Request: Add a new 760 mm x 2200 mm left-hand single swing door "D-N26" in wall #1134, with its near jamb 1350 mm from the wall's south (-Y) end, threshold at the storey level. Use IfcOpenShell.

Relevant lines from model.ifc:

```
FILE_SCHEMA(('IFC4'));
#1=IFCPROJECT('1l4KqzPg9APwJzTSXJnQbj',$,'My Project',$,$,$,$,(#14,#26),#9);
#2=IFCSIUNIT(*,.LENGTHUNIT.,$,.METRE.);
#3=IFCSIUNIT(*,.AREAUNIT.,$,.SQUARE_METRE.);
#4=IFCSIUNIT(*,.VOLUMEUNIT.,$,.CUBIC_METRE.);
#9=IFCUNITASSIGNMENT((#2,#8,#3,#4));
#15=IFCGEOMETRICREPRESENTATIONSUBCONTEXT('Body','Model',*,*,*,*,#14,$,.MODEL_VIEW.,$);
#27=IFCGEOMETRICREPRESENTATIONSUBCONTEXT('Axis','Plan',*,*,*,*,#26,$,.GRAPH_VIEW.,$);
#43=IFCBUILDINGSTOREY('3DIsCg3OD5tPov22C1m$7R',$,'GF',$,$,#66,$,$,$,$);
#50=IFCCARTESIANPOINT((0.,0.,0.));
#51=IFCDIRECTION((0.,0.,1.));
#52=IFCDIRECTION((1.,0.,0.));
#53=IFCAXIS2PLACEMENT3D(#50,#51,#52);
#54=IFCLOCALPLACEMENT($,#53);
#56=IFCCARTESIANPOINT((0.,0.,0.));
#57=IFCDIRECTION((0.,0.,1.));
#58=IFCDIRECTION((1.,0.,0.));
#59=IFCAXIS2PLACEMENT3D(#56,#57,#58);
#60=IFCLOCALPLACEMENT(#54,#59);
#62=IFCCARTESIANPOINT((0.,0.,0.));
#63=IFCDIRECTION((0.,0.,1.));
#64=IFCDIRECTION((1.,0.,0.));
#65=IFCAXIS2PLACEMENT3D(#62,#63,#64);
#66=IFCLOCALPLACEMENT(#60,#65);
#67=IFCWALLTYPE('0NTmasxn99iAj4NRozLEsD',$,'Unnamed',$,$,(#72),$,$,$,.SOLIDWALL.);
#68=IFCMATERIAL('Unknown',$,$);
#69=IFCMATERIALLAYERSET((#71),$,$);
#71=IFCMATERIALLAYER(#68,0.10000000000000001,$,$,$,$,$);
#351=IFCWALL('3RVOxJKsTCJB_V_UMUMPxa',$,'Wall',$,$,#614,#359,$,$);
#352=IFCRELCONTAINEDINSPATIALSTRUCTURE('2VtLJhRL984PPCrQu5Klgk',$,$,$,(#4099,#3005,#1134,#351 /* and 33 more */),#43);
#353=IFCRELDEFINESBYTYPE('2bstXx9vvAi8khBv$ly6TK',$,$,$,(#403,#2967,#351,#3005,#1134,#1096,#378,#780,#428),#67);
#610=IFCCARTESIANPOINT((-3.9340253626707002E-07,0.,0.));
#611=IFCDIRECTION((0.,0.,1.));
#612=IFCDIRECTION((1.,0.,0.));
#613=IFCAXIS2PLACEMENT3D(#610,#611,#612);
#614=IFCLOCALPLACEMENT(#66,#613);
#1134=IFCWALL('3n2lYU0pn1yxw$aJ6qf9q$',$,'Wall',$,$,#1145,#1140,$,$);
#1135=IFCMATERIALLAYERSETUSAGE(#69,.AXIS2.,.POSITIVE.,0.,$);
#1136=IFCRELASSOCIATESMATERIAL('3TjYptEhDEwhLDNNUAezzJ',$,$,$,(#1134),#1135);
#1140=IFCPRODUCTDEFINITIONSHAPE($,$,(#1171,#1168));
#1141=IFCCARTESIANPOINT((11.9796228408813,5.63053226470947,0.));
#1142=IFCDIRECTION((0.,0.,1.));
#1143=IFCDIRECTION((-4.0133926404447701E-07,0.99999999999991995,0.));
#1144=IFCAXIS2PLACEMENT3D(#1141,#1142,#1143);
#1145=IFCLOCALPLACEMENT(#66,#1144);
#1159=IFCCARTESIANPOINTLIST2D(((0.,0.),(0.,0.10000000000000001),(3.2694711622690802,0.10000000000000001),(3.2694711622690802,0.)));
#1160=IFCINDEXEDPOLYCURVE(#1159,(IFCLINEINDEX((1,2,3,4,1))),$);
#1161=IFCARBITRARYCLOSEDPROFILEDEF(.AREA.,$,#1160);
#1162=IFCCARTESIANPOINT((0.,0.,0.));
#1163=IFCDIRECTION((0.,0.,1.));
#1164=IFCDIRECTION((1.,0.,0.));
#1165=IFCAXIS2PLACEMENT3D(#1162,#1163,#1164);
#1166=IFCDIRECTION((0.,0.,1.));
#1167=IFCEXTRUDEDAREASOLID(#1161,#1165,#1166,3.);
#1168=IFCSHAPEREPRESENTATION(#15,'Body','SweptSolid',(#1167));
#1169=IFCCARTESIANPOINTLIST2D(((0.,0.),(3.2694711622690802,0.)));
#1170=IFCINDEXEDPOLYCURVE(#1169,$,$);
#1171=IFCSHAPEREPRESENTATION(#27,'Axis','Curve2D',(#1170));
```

```python
import numpy as np
import ifcopenshell
import ifcopenshell.api.feature
import ifcopenshell.api.geometry
import ifcopenshell.api.root
import ifcopenshell.api.spatial
import ifcopenshell.geom
import ifcopenshell.util.element
import ifcopenshell.util.placement
import ifcopenshell.util.representation
import ifcopenshell.util.shape
import ifcopenshell.util.unit

model = ifcopenshell.open("model.ifc")
unit_scale = ifcopenshell.util.unit.calculate_unit_scale(model)
settings = ifcopenshell.geom.settings()


def volume(element):
    """Net volume in cubic metres, openings subtracted."""
    shape = ifcopenshell.geom.create_shape(settings, element)
    return ifcopenshell.util.shape.get_volume(shape.geometry)


wall = model.by_guid("3n2lYU0pn1yxw$aJ6qf9q$")
storey = ifcopenshell.util.element.get_container(wall, ifc_class="IfcBuildingStorey")
context = ifcopenshell.util.representation.get_context(model, "Model", "Body", "MODEL_VIEW")
before = volume(wall)

width, height, from_end, sill = 0.76, 2.2, 1.35, 0.0  # metres

# The wall runs along its own X axis, and the end named is its -X end.
wall_shape = ifcopenshell.geom.create_shape(settings, wall)
x, y, z = ifcopenshell.util.shape.get_vertices(wall_shape.geometry).T
start = x.min() + from_end
face, thickness = float(y.min()), float(y.max() - y.min())
wall_matrix = ifcopenshell.util.placement.get_local_placement(wall.ObjectPlacement)
level = ifcopenshell.util.placement.get_local_placement(storey.ObjectPlacement)[2, 3]


def in_wall(x, y):
    """Placement at x, y metres in the wall's axes, at sill height."""
    matrix = wall_matrix.copy()
    matrix[:, 3] = wall_matrix @ np.array([x / unit_scale, y / unit_scale, 0.0, 1.0])
    matrix[2, 3] = level + sill / unit_scale
    return matrix


# Opening: a box that overshoots both wall faces by 50 mm.
opening = ifcopenshell.api.root.create_entity(model, ifc_class="IfcOpeningElement", predefined_type="OPENING")
box = ifcopenshell.api.geometry.add_wall_representation(
    model, context=context, length=width, height=height, thickness=thickness + 0.1
)
ifcopenshell.api.geometry.assign_representation(model, product=opening, representation=box)
ifcopenshell.api.geometry.edit_object_placement(model, product=opening, matrix=in_wall(start, face - 0.05), is_si=False)
ifcopenshell.api.feature.add_feature(model, feature=opening, element=wall)

door = ifcopenshell.api.root.create_entity(model, ifc_class="IfcDoor", name="D-N26", predefined_type="DOOR")
door.OverallWidth, door.OverallHeight = width / unit_scale, height / unit_scale
door.OperationType = "SINGLE_SWING_LEFT"
body = ifcopenshell.api.geometry.add_door_representation(
    model,
    context=context,
    overall_width=door.OverallWidth,
    overall_height=door.OverallHeight,
    operation_type="SINGLE_SWING_LEFT",
    lining_properties={"LiningDepth": thickness / unit_scale, "ThresholdDepth": thickness / unit_scale},
)
ifcopenshell.api.geometry.assign_representation(model, product=door, representation=body)
ifcopenshell.api.spatial.assign_container(model, products=[door], relating_structure=storey)
ifcopenshell.api.feature.add_filling(model, opening=opening, element=door)

# The lining spans the wall, so the door starts at the wall face.
ifcopenshell.api.geometry.edit_object_placement(model, product=door, matrix=in_wall(start, face), is_si=False)

after = volume(wall)

print(f"wall volume {before:.3f} -> {after:.3f} m3")

model.write("model_edited.ifc")
```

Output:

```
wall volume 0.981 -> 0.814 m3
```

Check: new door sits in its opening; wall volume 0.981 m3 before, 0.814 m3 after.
